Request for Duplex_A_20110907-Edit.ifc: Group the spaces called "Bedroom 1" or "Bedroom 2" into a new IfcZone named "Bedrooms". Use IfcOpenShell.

First a look at what the model holds.

```python
import ifcopenshell

model = ifcopenshell.open("Duplex_A_20110907-Edit.ifc")
print(model.schema)
seen = {}
for space in model.by_type("IfcSpace"):
    seen[space.LongName] = seen.get(space.LongName, 0) + 1
for name, count in sorted(seen.items(), key=str):
    print(count, "x", name)
print("zones:", [z.Name for z in model.by_type("IfcZone")][:20])
```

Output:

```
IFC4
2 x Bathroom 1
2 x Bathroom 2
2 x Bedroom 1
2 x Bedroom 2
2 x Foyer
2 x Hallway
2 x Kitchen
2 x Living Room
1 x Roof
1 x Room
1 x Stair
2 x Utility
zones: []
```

```python
import ifcopenshell
import ifcopenshell.api.group
import ifcopenshell.api.root

model = ifcopenshell.open("Duplex_A_20110907-Edit.ifc")

names = {"Bedroom 1", "Bedroom 2"}
spaces = [s for s in model.by_type("IfcSpace") if s.LongName in names]

zone = ifcopenshell.api.root.create_entity(model, ifc_class="IfcZone", name="Bedrooms")
ifcopenshell.api.group.assign_group(model, products=spaces, group=zone)
print(len(spaces), "spaces in", zone.Name)

model.write("Duplex_A_20110907-Edit_rev.ifc")
```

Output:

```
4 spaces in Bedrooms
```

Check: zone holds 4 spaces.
